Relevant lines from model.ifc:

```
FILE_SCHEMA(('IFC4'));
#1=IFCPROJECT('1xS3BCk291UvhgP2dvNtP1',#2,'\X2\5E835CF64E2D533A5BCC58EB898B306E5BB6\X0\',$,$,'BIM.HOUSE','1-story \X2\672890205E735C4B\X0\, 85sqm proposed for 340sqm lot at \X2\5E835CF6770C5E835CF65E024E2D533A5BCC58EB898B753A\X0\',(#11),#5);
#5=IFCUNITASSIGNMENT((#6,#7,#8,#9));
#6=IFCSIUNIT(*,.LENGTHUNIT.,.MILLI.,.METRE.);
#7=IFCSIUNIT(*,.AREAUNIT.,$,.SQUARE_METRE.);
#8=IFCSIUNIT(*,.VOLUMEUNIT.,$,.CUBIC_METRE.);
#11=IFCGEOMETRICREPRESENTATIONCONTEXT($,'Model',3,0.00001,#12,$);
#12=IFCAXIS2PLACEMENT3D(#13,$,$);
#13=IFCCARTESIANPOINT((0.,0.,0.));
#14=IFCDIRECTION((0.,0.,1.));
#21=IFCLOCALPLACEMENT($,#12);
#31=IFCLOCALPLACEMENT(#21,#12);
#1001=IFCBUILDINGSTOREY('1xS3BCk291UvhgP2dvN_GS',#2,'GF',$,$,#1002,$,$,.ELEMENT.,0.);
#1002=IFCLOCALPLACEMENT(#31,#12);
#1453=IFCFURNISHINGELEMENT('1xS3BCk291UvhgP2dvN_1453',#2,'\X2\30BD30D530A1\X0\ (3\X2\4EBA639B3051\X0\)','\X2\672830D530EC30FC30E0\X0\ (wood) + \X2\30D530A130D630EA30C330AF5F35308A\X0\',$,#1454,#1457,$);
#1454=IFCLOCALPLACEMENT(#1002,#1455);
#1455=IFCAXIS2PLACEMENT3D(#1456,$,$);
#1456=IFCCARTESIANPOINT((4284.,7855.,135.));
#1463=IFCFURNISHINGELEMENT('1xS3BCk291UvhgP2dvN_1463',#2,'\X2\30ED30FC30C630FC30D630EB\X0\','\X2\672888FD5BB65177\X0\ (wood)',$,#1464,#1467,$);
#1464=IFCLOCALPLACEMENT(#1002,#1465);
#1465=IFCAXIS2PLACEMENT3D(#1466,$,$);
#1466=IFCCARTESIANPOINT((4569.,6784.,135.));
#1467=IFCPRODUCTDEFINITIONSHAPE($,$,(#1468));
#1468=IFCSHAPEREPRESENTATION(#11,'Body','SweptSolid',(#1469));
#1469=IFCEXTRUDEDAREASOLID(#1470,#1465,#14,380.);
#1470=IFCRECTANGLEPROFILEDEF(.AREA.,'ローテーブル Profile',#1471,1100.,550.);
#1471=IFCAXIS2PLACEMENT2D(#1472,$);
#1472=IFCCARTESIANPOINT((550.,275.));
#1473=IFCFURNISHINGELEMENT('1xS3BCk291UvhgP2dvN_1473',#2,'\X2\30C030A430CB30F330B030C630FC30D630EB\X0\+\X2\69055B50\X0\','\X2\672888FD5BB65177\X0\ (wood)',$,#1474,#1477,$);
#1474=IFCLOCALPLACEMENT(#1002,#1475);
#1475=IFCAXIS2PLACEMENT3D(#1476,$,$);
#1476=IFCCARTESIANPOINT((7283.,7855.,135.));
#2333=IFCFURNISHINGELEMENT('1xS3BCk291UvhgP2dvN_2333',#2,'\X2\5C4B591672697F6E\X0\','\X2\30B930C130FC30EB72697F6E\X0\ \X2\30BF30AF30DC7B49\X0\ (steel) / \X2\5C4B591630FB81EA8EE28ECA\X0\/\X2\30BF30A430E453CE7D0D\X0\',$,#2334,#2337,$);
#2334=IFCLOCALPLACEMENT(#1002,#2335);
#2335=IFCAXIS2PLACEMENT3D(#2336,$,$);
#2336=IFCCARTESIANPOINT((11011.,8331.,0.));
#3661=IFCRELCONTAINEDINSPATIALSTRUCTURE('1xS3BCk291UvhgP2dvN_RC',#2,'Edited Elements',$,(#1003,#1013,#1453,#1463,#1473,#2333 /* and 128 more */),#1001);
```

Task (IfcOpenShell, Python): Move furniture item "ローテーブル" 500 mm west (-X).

```python
import ifcopenshell
import ifcopenshell.api.geometry
import ifcopenshell.util.placement
import ifcopenshell.util.unit

model = ifcopenshell.open("model.ifc")
unit_scale = ifcopenshell.util.unit.calculate_unit_scale(model)

item = model.by_guid("1xS3BCk291UvhgP2dvN_1463")
matrix = ifcopenshell.util.placement.get_local_placement(item.ObjectPlacement)
matrix[0, 3] -= 0.5 / unit_scale
ifcopenshell.api.geometry.edit_object_placement(model, product=item, matrix=matrix, is_si=False)

print(ifcopenshell.util.placement.get_local_placement(item.ObjectPlacement).round(3) + 0.0)

model.write("model_edited.ifc")
```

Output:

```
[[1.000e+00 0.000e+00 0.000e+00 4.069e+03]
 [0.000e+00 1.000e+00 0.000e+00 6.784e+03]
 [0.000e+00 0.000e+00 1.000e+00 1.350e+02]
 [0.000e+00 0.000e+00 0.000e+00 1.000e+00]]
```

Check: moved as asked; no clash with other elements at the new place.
